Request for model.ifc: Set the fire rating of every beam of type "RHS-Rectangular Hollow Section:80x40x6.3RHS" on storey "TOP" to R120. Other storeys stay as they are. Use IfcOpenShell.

First a look at what the model holds.

```python
import ifcopenshell
import ifcopenshell.util.element

model = ifcopenshell.open("model.ifc")
print(model.schema)
storey = next(s for s in model.by_type("IfcBuildingStorey") if s.Name == "TOP")
beams = [e for e in ifcopenshell.util.element.get_decomposition(storey) if e.is_a("IfcBeam")]
seen = {}
for e in beams:
    element_type = ifcopenshell.util.element.get_type(e)
    key = (element_type.Name if element_type != e and element_type else None, ifcopenshell.util.element.get_pset(e, "Pset_BeamCommon", "FireRating"))
    seen[key] = seen.get(key, 0) + 1
for (name, value), count in sorted(seen.items(), key=str):
    print(count, "x", name, "|", value)
```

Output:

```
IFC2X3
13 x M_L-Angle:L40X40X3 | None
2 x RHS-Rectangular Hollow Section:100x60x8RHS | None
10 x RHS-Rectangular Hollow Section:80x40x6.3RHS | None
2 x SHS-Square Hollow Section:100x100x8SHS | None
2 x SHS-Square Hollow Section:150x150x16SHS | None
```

```python
import ifcopenshell
import ifcopenshell.api.pset
import ifcopenshell.util.element

model = ifcopenshell.open("model.ifc")

storey = next(s for s in model.by_type("IfcBuildingStorey") if s.Name == "TOP")
beams = [e for e in ifcopenshell.util.element.get_decomposition(storey) if e.is_a("IfcBeam")]

count = 0
for e in beams:
    element_type = ifcopenshell.util.element.get_type(e)
    if element_type in (None, e) or element_type.Name != "RHS-Rectangular Hollow Section:80x40x6.3RHS":
        continue
    # add_pset returns the element's existing set when there is one.
    pset = ifcopenshell.api.pset.add_pset(model, product=e, name="Pset_BeamCommon")
    ifcopenshell.api.pset.edit_pset(model, pset=pset, properties={"FireRating": "R120"})
    count += 1

print(count, "beams updated")

model.write("model_rev.ifc")
```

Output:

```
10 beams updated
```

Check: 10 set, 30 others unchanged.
